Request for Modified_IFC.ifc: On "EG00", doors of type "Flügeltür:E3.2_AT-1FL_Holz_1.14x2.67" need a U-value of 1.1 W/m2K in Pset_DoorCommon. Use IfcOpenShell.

First a look at what the model holds.

```python
import ifcopenshell
import ifcopenshell.util.element

model = ifcopenshell.open("Modified_IFC.ifc")
print(model.schema)
storey = next(s for s in model.by_type("IfcBuildingStorey") if s.Name == "EG00")
doors = [e for e in ifcopenshell.util.element.get_decomposition(storey) if e.is_a("IfcDoor")]
seen = {}
for e in doors:
    element_type = ifcopenshell.util.element.get_type(e)
    key = (element_type.Name if element_type != e and element_type else None, ifcopenshell.util.element.get_pset(e, "Pset_DoorCommon", "ThermalTransmittance"))
    seen[key] = seen.get(key, 0) + 1
for (name, value), count in sorted(seen.items(), key=str):
    print(count, "x", name, "|", value)
```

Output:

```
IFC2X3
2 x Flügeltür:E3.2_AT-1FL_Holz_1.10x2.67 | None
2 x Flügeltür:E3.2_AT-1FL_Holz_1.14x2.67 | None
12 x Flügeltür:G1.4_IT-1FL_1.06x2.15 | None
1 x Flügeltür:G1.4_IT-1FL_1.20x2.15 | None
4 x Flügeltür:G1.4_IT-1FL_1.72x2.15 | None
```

```python
import ifcopenshell
import ifcopenshell.api.pset
import ifcopenshell.util.element

model = ifcopenshell.open("Modified_IFC.ifc")

storey = next(s for s in model.by_type("IfcBuildingStorey") if s.Name == "EG00")
doors = [e for e in ifcopenshell.util.element.get_decomposition(storey) if e.is_a("IfcDoor")]

count = 0
for e in doors:
    element_type = ifcopenshell.util.element.get_type(e)
    if element_type in (None, e) or element_type.Name != "Flügeltür:E3.2_AT-1FL_Holz_1.14x2.67":
        continue
    # add_pset returns the element's existing set when there is one.
    pset = ifcopenshell.api.pset.add_pset(model, product=e, name="Pset_DoorCommon")
    ifcopenshell.api.pset.edit_pset(model, pset=pset, properties={"ThermalTransmittance": 1.1})
    count += 1

print(count, "doors updated")

model.write("Modified_IFC_rev.ifc")
```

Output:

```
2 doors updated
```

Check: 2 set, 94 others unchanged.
